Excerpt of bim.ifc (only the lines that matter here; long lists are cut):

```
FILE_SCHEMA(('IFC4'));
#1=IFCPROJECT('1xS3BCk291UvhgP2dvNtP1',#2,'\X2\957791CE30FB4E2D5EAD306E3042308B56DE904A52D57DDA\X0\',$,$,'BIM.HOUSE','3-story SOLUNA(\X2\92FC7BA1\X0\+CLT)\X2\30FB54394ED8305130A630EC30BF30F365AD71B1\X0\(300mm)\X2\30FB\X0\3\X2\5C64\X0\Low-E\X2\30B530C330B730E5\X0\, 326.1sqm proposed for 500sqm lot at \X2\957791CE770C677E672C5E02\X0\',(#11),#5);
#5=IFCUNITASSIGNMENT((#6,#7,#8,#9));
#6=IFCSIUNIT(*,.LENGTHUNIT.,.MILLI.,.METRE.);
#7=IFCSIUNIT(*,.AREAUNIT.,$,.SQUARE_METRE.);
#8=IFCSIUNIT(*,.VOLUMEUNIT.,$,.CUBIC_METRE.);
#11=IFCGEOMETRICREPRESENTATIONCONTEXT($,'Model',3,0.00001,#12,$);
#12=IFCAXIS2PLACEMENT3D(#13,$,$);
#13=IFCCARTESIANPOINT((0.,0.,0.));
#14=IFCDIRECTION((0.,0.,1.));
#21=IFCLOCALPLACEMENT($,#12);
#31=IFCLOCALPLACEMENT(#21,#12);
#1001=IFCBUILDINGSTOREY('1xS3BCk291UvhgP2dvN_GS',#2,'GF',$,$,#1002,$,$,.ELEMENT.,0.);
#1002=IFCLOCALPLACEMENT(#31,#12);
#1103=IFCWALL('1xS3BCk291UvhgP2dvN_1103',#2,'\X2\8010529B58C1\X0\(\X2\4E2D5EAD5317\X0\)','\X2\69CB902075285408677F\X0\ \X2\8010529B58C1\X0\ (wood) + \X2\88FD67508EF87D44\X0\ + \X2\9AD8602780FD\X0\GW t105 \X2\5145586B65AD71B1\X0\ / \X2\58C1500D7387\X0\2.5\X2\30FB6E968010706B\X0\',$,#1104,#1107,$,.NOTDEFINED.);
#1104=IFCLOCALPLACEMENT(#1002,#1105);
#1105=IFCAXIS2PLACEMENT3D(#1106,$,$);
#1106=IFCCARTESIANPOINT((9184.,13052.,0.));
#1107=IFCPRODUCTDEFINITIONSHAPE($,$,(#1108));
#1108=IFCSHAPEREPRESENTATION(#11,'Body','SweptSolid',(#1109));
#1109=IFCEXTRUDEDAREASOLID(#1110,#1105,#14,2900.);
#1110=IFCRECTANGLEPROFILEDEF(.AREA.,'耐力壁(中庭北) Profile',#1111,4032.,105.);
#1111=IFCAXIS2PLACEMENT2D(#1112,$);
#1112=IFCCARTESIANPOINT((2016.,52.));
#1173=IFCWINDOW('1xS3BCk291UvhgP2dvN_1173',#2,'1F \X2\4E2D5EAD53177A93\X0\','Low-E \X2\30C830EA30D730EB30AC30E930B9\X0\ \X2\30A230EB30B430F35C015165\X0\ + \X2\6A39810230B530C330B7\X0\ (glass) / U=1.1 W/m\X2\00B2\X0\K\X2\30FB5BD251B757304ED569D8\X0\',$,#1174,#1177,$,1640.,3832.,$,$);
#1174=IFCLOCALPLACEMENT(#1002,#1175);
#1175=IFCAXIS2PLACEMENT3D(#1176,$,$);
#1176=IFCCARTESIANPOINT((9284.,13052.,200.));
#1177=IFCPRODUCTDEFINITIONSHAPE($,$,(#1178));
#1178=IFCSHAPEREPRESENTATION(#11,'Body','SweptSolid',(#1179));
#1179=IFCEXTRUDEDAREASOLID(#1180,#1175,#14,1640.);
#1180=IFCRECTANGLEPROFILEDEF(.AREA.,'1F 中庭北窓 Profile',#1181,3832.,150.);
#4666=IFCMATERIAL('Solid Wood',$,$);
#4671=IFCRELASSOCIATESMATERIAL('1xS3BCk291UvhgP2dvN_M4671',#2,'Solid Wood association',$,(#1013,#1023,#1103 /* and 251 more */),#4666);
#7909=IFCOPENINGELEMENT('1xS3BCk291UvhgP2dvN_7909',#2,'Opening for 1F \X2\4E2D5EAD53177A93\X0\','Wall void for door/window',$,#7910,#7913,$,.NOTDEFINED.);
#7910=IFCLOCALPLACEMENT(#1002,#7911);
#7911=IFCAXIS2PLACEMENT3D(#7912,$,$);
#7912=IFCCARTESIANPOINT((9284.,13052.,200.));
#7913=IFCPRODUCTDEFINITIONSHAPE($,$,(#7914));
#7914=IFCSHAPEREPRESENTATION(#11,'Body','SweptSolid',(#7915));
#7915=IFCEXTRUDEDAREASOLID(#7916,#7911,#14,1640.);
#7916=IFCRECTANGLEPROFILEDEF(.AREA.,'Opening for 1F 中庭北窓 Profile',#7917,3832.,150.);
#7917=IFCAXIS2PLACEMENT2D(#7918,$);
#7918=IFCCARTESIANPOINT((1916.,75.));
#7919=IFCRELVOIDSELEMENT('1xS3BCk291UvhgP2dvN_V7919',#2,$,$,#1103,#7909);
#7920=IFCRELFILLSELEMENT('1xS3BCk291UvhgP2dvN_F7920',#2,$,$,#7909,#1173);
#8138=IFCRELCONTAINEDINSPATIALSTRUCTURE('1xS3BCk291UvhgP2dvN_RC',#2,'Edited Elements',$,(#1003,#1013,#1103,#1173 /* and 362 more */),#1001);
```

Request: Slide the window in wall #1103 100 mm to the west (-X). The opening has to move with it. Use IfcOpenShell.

```python
import ifcopenshell
import ifcopenshell.api.geometry
import ifcopenshell.util.placement
import ifcopenshell.util.unit

model = ifcopenshell.open("bim.ifc")
unit_scale = ifcopenshell.util.unit.calculate_unit_scale(model)

window = model.by_guid("1xS3BCk291UvhgP2dvN_1173")
opening = window.FillsVoids[0].RelatingOpeningElement
wall = opening.VoidsElements[0].RelatingBuildingElement

wall_matrix = ifcopenshell.util.placement.get_local_placement(wall.ObjectPlacement)
shift = wall_matrix[:3, 0] * -0.1 / unit_scale
before = ifcopenshell.util.placement.get_local_placement(window.ObjectPlacement)[:3, 3].copy()

# The window is not placed relative to its opening, so move both.
for product in (opening, window):
    matrix = ifcopenshell.util.placement.get_local_placement(product.ObjectPlacement)
    matrix[:3, 3] += shift
    ifcopenshell.api.geometry.edit_object_placement(model, product=product, matrix=matrix, is_si=False)

after = ifcopenshell.util.placement.get_local_placement(window.ObjectPlacement)[:3, 3]
print("window moved by", (after - before).round(3) + 0.0)

model.write("bim_updated.ifc")
```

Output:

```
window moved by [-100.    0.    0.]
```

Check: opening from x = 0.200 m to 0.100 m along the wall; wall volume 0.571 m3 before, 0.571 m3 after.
